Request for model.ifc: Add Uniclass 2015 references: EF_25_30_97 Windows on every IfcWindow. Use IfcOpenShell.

First a look at what the model holds.

```python
import ifcopenshell

model = ifcopenshell.open("model.ifc")
print(model.schema)
print("classifications:", [c.Name for c in model.by_type("IfcClassification")])
for ifc_class in ("IfcDoor", "IfcRoof", "IfcStair", "IfcWall", "IfcWindow"):
    print(ifc_class, len(model.by_type(ifc_class)))
```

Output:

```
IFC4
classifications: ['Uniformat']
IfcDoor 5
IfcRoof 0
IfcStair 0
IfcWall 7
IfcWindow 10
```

```python
import ifcopenshell
import ifcopenshell.api.classification

model = ifcopenshell.open("model.ifc")

system = ifcopenshell.api.classification.add_classification(model, classification="Uniclass 2015")

codes = {
    "IfcWindow": ("EF_25_30_97", "Windows"),
}
for ifc_class, (code, name) in codes.items():
    products = model.by_type(ifc_class)
    ifcopenshell.api.classification.add_reference(
        model, products=products, classification=system, identification=code, name=name
    )
    print(code, len(products))

model.write("model_edited.ifc")
```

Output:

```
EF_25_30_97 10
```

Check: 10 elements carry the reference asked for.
